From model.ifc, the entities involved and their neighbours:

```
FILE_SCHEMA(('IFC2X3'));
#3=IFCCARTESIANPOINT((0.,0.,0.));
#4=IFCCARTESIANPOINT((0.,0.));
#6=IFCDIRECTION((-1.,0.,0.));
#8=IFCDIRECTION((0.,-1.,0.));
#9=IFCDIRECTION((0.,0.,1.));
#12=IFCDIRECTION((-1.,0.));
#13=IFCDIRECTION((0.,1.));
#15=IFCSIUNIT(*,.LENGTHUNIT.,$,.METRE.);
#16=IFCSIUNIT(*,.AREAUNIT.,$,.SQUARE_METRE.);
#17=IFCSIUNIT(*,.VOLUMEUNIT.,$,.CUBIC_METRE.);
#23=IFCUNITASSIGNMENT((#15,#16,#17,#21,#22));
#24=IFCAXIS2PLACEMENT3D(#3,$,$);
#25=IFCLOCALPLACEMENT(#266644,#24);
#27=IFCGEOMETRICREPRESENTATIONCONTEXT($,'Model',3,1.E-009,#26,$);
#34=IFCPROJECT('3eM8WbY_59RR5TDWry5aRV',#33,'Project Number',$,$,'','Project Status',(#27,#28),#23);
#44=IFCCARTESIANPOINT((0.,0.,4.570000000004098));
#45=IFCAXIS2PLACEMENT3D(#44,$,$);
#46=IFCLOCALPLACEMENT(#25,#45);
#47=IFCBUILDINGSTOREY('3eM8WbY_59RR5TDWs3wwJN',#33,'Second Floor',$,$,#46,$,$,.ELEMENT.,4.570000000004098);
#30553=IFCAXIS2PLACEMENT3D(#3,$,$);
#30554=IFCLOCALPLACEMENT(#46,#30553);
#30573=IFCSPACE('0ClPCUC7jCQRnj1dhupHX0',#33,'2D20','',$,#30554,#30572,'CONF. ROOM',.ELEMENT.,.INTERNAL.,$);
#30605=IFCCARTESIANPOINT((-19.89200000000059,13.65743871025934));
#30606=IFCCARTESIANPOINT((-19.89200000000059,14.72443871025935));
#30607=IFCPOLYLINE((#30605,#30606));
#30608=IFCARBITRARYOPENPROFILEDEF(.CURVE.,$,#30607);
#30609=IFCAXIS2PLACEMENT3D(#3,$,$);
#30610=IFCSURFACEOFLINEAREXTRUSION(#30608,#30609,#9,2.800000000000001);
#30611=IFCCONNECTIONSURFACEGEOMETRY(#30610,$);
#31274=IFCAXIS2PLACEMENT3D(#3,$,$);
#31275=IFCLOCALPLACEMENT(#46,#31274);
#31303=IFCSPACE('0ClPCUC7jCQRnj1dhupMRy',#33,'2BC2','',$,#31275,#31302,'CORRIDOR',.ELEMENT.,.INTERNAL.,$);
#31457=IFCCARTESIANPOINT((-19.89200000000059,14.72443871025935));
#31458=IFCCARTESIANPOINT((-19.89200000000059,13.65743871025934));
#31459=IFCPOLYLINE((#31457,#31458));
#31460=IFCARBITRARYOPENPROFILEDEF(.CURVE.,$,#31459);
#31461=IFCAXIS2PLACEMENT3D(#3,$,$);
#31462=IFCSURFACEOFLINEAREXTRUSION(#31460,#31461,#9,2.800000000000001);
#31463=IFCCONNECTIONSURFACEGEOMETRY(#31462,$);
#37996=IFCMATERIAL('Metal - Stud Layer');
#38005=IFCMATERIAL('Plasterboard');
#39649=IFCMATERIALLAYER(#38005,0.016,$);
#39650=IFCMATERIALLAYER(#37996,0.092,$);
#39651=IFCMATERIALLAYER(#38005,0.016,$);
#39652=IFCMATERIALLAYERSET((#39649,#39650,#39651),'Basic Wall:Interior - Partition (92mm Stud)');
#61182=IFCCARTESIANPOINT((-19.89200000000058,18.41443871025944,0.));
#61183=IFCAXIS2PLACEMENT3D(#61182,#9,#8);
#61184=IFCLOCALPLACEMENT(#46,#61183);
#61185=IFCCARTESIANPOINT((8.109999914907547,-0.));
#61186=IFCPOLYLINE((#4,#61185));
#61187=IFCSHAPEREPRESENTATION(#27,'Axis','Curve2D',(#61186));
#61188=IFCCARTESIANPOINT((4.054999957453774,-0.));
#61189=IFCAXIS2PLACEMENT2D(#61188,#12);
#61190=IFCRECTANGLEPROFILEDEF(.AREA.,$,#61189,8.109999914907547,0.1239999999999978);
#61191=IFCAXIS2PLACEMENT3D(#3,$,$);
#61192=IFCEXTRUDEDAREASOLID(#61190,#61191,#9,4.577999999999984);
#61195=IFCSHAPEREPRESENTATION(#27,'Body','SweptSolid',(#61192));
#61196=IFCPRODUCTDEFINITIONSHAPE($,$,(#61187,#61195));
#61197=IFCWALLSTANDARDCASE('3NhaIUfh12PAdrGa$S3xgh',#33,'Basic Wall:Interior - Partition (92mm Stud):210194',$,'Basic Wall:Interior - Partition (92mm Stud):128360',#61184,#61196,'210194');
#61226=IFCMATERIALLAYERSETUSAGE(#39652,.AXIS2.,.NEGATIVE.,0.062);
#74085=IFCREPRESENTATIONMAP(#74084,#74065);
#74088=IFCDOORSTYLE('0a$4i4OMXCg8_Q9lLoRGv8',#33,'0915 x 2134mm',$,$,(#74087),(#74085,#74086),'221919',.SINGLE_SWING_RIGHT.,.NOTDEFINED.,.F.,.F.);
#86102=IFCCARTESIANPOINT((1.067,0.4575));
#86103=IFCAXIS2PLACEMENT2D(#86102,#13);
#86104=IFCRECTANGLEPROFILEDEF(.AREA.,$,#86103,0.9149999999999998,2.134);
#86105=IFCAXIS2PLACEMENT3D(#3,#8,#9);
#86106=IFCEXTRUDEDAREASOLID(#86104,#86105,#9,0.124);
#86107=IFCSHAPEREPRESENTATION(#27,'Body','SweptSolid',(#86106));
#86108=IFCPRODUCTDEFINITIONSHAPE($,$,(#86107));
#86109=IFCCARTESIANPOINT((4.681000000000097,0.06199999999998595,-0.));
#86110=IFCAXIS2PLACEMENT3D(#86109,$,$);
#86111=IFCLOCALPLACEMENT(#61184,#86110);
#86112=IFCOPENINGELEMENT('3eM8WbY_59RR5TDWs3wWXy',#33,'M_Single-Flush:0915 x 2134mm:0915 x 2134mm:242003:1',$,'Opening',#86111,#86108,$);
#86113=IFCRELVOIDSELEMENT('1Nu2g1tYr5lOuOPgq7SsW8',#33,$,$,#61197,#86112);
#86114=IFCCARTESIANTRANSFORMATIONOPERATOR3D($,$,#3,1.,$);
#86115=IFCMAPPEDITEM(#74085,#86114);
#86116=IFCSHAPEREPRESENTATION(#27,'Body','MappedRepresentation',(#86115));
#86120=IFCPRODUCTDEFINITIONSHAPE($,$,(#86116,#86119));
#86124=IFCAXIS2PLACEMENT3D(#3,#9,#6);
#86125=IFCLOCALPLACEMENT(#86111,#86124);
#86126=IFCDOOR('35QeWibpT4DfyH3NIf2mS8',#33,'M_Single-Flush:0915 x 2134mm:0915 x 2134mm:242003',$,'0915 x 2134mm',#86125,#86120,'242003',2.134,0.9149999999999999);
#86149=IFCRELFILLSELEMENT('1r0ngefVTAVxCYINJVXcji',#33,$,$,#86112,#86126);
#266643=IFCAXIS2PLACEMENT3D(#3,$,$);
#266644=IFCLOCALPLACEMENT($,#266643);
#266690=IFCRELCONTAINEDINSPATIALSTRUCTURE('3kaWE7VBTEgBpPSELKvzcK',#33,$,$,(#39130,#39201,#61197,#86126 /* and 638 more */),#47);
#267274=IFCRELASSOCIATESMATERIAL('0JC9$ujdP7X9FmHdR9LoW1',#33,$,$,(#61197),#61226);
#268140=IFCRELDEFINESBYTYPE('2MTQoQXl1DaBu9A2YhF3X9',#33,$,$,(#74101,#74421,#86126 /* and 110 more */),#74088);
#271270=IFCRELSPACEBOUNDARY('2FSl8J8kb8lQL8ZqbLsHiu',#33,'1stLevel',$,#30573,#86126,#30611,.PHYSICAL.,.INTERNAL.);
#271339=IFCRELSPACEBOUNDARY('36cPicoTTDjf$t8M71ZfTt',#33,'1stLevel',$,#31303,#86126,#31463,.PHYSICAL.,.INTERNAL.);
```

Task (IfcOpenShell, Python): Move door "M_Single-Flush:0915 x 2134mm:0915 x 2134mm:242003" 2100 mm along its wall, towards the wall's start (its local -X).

```python
import numpy as np
import ifcopenshell
import ifcopenshell.api.geometry
import ifcopenshell.util.placement

model = ifcopenshell.open("model.ifc")

door = model.by_guid("35QeWibpT4DfyH3NIf2mS8")
opening = door.FillsVoids[0].RelatingOpeningElement
wall = opening.VoidsElements[0].RelatingBuildingElement

wall_matrix = ifcopenshell.util.placement.get_local_placement(wall.ObjectPlacement)
shift = wall_matrix[:3, 0] * -2.1
before = ifcopenshell.util.placement.get_local_placement(door.ObjectPlacement)[:3, 3].copy()

# The door is placed relative to its opening, so it follows when the opening moves.
matrix = ifcopenshell.util.placement.get_local_placement(opening.ObjectPlacement)
matrix[:3, 3] += shift
ifcopenshell.api.geometry.edit_object_placement(
    model, product=opening, matrix=matrix, is_si=False, should_transform_children=True
)

# Space boundary surfaces are stored in each space's coordinates; move them too.
for rel in door.ProvidesBoundaries:
    if not rel.ConnectionGeometry:
        continue
    surface = rel.ConnectionGeometry.SurfaceOnRelatingElement
    space_matrix = ifcopenshell.util.placement.get_local_placement(rel.RelatingSpace.ObjectPlacement)
    point = np.array(surface.Position.Location.Coordinates) + space_matrix[:3, :3].T @ shift
    surface.Position = model.createIfcAxis2Placement3D(
        model.createIfcCartesianPoint(point.tolist()), surface.Position.Axis, surface.Position.RefDirection
    )

after = ifcopenshell.util.placement.get_local_placement(door.ObjectPlacement)[:3, 3]
print("door moved by", (after - before).round(3) + 0.0)

model.write("model_updated.ifc")
```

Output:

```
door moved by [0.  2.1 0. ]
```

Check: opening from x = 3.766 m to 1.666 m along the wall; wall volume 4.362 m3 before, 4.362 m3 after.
